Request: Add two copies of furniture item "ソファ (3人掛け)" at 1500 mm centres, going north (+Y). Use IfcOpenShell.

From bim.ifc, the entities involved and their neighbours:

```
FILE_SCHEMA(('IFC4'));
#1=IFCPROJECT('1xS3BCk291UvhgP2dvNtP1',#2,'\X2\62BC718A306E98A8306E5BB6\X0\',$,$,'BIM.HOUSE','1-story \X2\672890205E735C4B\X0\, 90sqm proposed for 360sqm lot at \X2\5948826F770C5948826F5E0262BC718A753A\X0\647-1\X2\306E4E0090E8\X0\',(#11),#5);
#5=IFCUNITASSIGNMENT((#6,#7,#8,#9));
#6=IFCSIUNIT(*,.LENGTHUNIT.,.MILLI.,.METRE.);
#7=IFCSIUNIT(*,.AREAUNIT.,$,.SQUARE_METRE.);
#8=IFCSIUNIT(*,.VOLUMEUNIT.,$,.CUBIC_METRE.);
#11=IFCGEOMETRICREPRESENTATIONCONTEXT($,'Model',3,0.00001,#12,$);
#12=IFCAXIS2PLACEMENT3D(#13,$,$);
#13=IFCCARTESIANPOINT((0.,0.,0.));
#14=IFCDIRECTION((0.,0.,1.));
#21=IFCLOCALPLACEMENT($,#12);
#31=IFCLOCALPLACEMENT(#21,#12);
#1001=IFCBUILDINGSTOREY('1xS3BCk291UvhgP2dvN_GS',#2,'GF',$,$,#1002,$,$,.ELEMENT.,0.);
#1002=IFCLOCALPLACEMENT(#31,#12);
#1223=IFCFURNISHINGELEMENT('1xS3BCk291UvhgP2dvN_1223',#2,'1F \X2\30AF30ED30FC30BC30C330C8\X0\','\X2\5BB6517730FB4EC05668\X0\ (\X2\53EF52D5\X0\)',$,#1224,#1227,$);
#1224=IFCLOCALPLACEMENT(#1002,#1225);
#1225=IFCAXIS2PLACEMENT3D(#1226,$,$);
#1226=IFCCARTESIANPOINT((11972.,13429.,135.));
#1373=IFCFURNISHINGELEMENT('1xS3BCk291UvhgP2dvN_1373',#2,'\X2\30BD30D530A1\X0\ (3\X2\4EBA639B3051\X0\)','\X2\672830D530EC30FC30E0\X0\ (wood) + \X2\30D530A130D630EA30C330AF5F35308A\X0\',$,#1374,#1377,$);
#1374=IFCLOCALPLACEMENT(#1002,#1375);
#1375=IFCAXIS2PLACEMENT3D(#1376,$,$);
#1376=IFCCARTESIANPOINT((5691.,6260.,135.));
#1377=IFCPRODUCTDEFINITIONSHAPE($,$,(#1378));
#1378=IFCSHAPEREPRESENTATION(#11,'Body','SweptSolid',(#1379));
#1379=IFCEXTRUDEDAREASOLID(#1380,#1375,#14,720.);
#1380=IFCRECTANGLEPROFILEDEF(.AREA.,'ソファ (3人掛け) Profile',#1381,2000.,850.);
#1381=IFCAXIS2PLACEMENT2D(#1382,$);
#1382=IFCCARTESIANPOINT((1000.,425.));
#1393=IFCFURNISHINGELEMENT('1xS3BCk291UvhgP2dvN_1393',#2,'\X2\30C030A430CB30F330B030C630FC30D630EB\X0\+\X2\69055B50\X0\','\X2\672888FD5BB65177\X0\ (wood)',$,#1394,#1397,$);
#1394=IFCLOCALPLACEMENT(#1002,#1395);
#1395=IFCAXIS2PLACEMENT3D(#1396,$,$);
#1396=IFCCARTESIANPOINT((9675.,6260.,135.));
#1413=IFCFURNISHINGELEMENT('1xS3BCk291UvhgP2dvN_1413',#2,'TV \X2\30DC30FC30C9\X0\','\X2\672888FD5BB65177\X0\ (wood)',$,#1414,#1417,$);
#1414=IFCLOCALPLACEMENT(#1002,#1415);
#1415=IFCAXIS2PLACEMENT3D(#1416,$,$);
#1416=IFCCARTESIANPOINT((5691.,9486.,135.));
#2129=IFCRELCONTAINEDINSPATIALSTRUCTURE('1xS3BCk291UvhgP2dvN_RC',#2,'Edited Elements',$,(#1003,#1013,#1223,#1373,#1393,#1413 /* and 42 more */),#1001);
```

```python
import numpy as np
import ifcopenshell
import ifcopenshell.api.geometry
import ifcopenshell.api.root
import ifcopenshell.util.element
import ifcopenshell.util.placement

model = ifcopenshell.open("bim.ifc")


def reuse_history(source, copy):
    """copy_class also copies each property set's owner history, people and application; keep the originals."""
    for rel in copy.IsDefinedBy:
        if rel.is_a("IfcRelDefinesByProperties") and (history := rel.RelatingPropertyDefinition.OwnerHistory):
            rel.RelatingPropertyDefinition.OwnerHistory = source.OwnerHistory
            ifcopenshell.util.element.remove_deep2(model, history)


source = model.by_guid("1xS3BCk291UvhgP2dvN_1373")
base = ifcopenshell.util.placement.get_local_placement(source.ObjectPlacement)
step = np.array([0.0, 1.0, 0.0]) * 1500.0

for i in range(1, 3):
    copy = ifcopenshell.api.root.copy_class(model, product=source)
    copy.Representation = ifcopenshell.util.element.copy_deep(
        model, source.Representation, exclude=["IfcGeometricRepresentationContext", "IfcRepresentationMap"]
    )
    reuse_history(source, copy)
    matrix = base.copy()
    matrix[:3, 3] += i * step
    print("added at", matrix[:3, 3].round(3) + 0.0)
    ifcopenshell.api.geometry.edit_object_placement(model, product=copy, matrix=matrix, is_si=False)

model.write("bim_edited.ifc")
```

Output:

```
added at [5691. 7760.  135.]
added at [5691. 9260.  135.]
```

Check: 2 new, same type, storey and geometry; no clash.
